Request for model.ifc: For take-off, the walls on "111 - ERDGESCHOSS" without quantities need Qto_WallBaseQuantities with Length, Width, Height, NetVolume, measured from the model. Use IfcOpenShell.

First a look at what the model holds.

```python
import ifcopenshell
import ifcopenshell.util.element
import ifcopenshell.util.unit

model = ifcopenshell.open("model.ifc")
print(model.schema)
for unit_type in ("LENGTHUNIT", "AREAUNIT", "VOLUMEUNIT"):
    print(unit_type, ifcopenshell.util.unit.calculate_unit_scale(model, unit_type))
storey = next(s for s in model.by_type("IfcBuildingStorey") if s.Name == "111 - ERDGESCHOSS")
walls = [e for e in ifcopenshell.util.element.get_decomposition(storey) if e.is_a("IfcWall")]
for e in sorted(walls, key=lambda e: e.id()):
    print(e.id(), e.is_a(), e.Name, list(ifcopenshell.util.element.get_psets(e, qtos_only=True)), sep=" | ")
```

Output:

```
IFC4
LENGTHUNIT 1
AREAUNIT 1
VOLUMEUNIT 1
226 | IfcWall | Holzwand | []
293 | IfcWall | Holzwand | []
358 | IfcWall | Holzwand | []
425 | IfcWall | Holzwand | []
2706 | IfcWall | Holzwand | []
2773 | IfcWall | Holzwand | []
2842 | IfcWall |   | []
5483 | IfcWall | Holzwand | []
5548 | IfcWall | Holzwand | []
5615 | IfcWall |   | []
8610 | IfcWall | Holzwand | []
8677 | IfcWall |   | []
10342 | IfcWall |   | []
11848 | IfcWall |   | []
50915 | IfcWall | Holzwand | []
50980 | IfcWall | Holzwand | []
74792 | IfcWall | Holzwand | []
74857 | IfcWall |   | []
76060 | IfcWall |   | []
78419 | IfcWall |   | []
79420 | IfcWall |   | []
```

```python
import ifcopenshell
import ifcopenshell.api.pset
import ifcopenshell.geom
import ifcopenshell.util.element
import ifcopenshell.util.shape
import ifcopenshell.util.unit

model = ifcopenshell.open("model.ifc")
unit_scale = ifcopenshell.util.unit.calculate_unit_scale(model)
volume_scale = ifcopenshell.util.unit.calculate_unit_scale(model, "VOLUMEUNIT")
settings = ifcopenshell.geom.settings()

storey = next(s for s in model.by_type("IfcBuildingStorey") if s.Name == "111 - ERDGESCHOSS")
walls = [e for e in ifcopenshell.util.element.get_decomposition(storey) if e.is_a("IfcWall")]

for e in sorted(walls, key=lambda e: e.id()):
    if ifcopenshell.util.element.get_psets(e, qtos_only=True, should_inherit=False):
        continue
    # Geometry comes back in metres, in the element's own axes.
    shape = ifcopenshell.geom.create_shape(settings, e)
    values = {
        "Length": ifcopenshell.util.shape.get_x(shape.geometry) / unit_scale,
        "Width": ifcopenshell.util.shape.get_y(shape.geometry) / unit_scale,
        "Height": ifcopenshell.util.shape.get_z(shape.geometry) / unit_scale,
        "NetVolume": ifcopenshell.util.shape.get_volume(shape.geometry) / volume_scale,
    }
    qto = ifcopenshell.api.pset.add_qto(model, product=e, name="Qto_WallBaseQuantities")
    ifcopenshell.api.pset.edit_qto(model, qto=qto, properties=values)
    print(e.id(), {k: round(v, 3) for k, v in values.items()})

model.write("model_rev.ifc")
```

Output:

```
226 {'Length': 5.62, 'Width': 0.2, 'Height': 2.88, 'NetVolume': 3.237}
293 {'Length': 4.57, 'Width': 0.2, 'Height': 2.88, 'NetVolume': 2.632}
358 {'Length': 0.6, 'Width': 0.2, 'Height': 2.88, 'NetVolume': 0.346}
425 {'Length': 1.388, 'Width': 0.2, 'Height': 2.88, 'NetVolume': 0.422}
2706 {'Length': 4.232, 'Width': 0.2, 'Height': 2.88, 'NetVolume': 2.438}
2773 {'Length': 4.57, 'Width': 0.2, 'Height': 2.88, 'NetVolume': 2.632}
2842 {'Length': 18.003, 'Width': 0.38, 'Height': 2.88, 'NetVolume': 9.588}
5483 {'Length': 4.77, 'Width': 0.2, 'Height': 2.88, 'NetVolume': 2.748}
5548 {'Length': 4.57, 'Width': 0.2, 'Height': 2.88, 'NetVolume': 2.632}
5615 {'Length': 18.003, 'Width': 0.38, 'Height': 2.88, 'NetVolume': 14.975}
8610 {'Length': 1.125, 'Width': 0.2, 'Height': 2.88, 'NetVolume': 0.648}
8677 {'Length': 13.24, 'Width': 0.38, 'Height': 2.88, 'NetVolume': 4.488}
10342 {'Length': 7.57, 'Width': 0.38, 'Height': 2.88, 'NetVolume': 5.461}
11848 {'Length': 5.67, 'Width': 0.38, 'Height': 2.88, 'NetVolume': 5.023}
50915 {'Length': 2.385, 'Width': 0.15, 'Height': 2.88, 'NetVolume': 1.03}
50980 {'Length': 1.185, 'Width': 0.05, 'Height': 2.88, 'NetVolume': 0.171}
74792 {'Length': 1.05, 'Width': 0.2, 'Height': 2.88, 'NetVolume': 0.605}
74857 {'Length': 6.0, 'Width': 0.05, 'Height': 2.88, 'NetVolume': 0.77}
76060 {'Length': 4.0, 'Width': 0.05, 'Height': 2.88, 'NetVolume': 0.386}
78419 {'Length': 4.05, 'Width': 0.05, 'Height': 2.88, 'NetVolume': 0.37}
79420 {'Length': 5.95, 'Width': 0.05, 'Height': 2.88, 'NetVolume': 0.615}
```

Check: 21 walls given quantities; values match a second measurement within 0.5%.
